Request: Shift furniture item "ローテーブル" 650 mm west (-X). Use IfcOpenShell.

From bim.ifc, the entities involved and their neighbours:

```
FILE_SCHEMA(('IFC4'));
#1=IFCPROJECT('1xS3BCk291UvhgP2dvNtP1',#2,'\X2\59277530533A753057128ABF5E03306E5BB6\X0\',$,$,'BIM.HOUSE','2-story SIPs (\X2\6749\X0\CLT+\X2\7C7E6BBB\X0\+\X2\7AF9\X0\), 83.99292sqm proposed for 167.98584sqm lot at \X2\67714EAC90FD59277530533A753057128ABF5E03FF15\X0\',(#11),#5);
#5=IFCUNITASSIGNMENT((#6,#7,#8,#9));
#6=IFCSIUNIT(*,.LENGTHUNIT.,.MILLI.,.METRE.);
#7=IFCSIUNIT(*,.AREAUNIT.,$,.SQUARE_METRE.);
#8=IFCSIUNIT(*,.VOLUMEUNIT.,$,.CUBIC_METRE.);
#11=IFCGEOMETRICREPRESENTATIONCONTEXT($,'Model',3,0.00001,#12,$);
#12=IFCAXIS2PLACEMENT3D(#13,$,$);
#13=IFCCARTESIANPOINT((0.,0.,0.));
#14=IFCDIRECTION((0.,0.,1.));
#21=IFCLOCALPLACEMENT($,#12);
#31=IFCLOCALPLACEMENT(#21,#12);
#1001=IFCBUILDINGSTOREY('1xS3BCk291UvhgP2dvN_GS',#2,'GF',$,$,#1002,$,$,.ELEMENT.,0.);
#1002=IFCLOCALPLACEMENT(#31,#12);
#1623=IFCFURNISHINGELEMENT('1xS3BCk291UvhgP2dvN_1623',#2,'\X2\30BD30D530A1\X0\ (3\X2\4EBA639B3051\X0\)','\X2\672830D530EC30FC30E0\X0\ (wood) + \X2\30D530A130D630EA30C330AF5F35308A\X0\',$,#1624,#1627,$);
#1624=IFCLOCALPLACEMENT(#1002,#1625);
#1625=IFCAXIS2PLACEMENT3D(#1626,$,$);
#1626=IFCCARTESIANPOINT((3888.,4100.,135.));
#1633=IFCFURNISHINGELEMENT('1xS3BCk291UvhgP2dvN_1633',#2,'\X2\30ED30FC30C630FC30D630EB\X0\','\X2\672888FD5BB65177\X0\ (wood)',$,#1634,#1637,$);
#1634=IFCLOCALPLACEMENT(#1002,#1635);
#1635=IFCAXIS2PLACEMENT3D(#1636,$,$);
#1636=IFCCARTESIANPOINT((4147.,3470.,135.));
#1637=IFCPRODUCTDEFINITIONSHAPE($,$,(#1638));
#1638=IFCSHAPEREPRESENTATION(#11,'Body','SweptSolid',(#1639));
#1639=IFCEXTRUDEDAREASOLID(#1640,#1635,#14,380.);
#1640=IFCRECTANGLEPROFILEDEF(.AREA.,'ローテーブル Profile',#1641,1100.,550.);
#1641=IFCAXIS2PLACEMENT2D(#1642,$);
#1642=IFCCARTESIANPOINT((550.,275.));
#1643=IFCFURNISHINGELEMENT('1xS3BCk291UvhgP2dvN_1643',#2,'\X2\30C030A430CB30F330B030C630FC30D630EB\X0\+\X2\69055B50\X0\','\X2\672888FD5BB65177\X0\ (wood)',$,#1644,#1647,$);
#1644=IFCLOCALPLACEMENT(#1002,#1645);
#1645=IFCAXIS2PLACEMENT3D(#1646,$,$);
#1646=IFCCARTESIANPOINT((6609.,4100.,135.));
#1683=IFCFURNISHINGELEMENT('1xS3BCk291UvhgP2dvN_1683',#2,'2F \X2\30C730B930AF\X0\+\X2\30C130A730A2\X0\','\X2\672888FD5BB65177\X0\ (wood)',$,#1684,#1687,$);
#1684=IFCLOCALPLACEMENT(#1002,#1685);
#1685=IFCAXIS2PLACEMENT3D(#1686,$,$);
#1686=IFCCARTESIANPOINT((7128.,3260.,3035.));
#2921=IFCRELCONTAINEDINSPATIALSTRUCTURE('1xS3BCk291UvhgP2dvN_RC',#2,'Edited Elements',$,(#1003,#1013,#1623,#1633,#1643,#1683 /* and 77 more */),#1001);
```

```python
import ifcopenshell
import ifcopenshell.api.geometry
import ifcopenshell.util.placement
import ifcopenshell.util.unit

model = ifcopenshell.open("bim.ifc")
unit_scale = ifcopenshell.util.unit.calculate_unit_scale(model)

item = model.by_guid("1xS3BCk291UvhgP2dvN_1633")
matrix = ifcopenshell.util.placement.get_local_placement(item.ObjectPlacement)
matrix[0, 3] -= 0.65 / unit_scale
ifcopenshell.api.geometry.edit_object_placement(model, product=item, matrix=matrix, is_si=False)

print(ifcopenshell.util.placement.get_local_placement(item.ObjectPlacement).round(3) + 0.0)

model.write("bim_rev.ifc")
```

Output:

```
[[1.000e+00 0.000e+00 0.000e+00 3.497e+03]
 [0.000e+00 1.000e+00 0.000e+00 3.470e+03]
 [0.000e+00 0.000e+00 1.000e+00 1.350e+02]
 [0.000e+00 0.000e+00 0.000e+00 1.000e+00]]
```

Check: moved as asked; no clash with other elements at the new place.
